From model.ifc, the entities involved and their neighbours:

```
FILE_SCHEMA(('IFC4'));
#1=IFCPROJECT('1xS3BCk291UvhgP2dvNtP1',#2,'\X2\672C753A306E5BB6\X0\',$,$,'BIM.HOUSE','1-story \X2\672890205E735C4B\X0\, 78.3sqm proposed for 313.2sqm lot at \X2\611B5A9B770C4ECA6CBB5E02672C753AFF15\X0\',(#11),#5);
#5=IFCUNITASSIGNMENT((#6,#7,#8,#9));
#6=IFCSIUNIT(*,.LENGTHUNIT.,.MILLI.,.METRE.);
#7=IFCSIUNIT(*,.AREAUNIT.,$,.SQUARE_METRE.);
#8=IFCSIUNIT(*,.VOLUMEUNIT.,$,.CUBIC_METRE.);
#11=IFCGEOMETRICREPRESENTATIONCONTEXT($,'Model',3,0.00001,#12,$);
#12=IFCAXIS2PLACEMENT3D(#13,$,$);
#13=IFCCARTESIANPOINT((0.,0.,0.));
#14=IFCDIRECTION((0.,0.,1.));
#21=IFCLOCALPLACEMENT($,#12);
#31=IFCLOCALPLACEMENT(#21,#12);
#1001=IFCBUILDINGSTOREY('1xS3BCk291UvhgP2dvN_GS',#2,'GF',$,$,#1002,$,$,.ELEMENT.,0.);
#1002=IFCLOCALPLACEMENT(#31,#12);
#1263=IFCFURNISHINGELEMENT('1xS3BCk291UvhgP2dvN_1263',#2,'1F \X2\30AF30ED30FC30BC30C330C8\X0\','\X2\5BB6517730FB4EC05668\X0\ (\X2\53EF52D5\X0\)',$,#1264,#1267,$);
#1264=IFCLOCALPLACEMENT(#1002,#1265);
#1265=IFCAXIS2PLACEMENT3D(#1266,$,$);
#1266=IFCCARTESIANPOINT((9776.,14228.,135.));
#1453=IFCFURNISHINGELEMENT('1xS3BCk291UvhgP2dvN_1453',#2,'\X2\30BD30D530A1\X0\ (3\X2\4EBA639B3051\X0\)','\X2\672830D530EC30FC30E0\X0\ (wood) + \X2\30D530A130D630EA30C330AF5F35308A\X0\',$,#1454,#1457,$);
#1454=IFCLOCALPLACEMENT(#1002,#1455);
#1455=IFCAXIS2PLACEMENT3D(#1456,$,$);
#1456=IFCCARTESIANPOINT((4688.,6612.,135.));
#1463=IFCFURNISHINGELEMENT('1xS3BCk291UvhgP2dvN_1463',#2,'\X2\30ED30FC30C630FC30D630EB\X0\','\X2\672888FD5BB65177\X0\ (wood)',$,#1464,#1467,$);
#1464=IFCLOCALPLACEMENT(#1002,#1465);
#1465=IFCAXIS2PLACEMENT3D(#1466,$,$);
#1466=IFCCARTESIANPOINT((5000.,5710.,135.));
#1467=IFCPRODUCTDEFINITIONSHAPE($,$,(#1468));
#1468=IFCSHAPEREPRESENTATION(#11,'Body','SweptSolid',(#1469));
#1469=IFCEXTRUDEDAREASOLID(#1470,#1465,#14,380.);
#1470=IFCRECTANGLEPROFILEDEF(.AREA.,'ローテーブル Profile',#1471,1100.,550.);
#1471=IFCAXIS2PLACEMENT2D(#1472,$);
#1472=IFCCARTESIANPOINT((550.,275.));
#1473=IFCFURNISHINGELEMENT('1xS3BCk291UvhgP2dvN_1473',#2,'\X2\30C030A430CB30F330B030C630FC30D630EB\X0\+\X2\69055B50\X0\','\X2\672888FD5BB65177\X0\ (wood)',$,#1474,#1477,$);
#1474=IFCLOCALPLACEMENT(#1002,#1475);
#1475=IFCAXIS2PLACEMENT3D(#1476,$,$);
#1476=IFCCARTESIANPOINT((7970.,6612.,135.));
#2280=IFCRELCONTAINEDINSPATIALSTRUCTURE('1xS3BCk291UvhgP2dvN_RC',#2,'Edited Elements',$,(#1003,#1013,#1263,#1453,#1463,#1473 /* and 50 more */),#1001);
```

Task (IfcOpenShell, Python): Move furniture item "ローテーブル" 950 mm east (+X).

```python
import ifcopenshell
import ifcopenshell.api.geometry
import ifcopenshell.util.placement

model = ifcopenshell.open("model.ifc")

item = model.by_guid("1xS3BCk291UvhgP2dvN_1463")
matrix = ifcopenshell.util.placement.get_local_placement(item.ObjectPlacement)
matrix[0, 3] += 950.0
ifcopenshell.api.geometry.edit_object_placement(model, product=item, matrix=matrix, is_si=False)

print(ifcopenshell.util.placement.get_local_placement(item.ObjectPlacement).round(3) + 0.0)

model.write("model_v2.ifc")
```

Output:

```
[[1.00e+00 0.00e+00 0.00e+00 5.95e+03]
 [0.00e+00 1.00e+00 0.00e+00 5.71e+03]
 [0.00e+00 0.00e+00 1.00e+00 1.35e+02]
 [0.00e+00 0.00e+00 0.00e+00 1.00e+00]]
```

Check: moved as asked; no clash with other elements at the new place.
